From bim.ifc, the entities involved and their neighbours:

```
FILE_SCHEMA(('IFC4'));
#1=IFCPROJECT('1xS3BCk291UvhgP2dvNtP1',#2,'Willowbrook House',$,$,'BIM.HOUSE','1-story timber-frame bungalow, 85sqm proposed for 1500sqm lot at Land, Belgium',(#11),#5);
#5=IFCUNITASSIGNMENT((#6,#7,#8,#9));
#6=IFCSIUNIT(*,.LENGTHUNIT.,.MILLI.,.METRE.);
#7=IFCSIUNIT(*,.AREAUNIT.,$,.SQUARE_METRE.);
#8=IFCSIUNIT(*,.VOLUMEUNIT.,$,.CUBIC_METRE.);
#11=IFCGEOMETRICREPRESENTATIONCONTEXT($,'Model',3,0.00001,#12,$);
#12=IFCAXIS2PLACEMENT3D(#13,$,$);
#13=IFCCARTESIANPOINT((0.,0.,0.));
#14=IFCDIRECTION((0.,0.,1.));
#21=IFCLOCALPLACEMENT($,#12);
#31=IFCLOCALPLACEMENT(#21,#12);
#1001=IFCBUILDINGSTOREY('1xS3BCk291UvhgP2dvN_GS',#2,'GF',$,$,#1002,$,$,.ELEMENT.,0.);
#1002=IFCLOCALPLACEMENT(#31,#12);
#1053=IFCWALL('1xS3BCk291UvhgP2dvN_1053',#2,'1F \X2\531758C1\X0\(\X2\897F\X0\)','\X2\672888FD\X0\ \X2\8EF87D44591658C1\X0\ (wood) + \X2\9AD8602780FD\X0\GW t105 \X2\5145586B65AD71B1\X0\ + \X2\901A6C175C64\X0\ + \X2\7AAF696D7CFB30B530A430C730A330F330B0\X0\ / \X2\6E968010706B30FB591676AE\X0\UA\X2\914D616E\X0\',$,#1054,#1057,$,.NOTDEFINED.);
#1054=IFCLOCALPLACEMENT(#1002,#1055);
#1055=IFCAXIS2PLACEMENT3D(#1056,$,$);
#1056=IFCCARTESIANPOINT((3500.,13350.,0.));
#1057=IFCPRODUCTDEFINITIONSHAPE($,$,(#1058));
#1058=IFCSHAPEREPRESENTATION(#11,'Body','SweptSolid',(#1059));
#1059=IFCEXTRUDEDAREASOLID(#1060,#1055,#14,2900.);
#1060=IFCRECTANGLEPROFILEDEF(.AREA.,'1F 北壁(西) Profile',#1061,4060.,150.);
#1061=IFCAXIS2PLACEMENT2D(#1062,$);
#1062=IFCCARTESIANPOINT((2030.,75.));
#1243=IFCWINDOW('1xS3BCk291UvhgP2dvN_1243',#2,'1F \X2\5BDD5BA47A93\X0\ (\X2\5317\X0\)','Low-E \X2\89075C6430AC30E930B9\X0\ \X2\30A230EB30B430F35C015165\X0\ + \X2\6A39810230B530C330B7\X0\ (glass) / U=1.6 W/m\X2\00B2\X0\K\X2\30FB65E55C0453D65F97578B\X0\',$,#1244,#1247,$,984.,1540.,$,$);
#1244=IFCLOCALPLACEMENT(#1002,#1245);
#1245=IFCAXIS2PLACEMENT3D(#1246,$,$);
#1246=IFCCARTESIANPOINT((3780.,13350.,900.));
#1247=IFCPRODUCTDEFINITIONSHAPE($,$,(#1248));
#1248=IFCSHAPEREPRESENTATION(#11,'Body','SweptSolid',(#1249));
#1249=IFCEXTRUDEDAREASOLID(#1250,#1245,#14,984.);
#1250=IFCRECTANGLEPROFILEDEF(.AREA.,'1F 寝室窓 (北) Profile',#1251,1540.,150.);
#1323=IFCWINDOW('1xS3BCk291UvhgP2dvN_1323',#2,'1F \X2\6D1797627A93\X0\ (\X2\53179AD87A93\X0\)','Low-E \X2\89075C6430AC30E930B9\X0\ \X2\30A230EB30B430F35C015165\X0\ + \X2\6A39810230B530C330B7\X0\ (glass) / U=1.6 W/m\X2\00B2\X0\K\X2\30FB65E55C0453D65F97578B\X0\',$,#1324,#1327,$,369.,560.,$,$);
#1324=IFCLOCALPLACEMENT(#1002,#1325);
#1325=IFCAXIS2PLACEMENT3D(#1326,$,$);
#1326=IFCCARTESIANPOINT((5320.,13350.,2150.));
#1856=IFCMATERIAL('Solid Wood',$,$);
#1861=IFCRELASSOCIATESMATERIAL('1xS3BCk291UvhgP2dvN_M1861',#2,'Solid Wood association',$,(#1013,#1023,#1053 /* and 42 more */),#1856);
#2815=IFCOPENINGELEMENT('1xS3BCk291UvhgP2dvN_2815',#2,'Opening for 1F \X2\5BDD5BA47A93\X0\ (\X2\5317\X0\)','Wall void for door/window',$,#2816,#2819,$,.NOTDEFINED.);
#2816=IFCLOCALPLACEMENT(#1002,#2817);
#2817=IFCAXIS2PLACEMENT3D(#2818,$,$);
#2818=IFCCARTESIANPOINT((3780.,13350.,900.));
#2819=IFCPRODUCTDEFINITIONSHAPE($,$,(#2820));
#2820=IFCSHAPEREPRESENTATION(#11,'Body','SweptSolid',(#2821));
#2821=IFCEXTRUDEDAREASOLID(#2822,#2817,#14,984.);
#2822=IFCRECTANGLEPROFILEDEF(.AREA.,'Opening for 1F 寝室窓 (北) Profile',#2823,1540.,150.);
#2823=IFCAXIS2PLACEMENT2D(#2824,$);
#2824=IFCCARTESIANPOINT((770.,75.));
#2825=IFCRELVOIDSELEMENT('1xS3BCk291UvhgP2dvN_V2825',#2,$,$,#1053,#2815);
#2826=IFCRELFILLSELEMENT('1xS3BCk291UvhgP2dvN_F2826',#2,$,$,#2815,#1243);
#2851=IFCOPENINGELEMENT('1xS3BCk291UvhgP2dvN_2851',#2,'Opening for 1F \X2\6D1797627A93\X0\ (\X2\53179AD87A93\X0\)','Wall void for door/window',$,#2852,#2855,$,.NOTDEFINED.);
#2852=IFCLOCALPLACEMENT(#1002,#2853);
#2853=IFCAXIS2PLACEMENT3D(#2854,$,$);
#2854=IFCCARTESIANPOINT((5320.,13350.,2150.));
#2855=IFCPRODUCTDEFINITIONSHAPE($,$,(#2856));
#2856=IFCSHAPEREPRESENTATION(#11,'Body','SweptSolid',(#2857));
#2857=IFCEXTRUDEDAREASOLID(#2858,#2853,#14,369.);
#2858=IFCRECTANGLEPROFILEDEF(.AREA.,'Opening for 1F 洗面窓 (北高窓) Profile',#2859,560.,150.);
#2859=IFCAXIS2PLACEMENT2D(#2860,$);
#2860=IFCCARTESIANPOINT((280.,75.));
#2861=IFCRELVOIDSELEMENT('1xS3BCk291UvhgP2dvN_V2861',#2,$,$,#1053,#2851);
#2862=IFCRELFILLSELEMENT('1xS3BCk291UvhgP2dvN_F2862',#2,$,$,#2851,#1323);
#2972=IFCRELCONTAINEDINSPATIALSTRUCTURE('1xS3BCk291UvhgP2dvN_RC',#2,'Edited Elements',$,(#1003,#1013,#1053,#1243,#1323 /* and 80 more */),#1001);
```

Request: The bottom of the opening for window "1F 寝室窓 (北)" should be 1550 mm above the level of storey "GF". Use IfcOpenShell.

```python
import numpy as np
import ifcopenshell
import ifcopenshell.api.geometry
import ifcopenshell.geom
import ifcopenshell.util.element
import ifcopenshell.util.placement
import ifcopenshell.util.shape
import ifcopenshell.util.unit

model = ifcopenshell.open("bim.ifc")
unit_scale = ifcopenshell.util.unit.calculate_unit_scale(model)

window = model.by_guid("1xS3BCk291UvhgP2dvN_1243")
opening = window.FillsVoids[0].RelatingOpeningElement
storey = ifcopenshell.util.element.get_container(window, ifc_class="IfcBuildingStorey")
level = ifcopenshell.util.placement.get_local_placement(storey.ObjectPlacement)[2, 3]

# The opening's origin need not be at the sill, so measure its lowest point.
shape = ifcopenshell.geom.create_shape(ifcopenshell.geom.settings(), opening)
bottom = ifcopenshell.util.shape.get_shape_bottom_elevation(shape, shape.geometry) / unit_scale
dz = level + 1550.0 - bottom

shift = np.array([0.0, 0.0, dz])
# The window is not placed relative to its opening, so move both.
for product in (opening, window):
    matrix = ifcopenshell.util.placement.get_local_placement(product.ObjectPlacement)
    matrix[:3, 3] += shift
    ifcopenshell.api.geometry.edit_object_placement(model, product=product, matrix=matrix, is_si=False)

print(f"moved by {dz * unit_scale:+.3f} m")

model.write("bim_edited.ifc")
```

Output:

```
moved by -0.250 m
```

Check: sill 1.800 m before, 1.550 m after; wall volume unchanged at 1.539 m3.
